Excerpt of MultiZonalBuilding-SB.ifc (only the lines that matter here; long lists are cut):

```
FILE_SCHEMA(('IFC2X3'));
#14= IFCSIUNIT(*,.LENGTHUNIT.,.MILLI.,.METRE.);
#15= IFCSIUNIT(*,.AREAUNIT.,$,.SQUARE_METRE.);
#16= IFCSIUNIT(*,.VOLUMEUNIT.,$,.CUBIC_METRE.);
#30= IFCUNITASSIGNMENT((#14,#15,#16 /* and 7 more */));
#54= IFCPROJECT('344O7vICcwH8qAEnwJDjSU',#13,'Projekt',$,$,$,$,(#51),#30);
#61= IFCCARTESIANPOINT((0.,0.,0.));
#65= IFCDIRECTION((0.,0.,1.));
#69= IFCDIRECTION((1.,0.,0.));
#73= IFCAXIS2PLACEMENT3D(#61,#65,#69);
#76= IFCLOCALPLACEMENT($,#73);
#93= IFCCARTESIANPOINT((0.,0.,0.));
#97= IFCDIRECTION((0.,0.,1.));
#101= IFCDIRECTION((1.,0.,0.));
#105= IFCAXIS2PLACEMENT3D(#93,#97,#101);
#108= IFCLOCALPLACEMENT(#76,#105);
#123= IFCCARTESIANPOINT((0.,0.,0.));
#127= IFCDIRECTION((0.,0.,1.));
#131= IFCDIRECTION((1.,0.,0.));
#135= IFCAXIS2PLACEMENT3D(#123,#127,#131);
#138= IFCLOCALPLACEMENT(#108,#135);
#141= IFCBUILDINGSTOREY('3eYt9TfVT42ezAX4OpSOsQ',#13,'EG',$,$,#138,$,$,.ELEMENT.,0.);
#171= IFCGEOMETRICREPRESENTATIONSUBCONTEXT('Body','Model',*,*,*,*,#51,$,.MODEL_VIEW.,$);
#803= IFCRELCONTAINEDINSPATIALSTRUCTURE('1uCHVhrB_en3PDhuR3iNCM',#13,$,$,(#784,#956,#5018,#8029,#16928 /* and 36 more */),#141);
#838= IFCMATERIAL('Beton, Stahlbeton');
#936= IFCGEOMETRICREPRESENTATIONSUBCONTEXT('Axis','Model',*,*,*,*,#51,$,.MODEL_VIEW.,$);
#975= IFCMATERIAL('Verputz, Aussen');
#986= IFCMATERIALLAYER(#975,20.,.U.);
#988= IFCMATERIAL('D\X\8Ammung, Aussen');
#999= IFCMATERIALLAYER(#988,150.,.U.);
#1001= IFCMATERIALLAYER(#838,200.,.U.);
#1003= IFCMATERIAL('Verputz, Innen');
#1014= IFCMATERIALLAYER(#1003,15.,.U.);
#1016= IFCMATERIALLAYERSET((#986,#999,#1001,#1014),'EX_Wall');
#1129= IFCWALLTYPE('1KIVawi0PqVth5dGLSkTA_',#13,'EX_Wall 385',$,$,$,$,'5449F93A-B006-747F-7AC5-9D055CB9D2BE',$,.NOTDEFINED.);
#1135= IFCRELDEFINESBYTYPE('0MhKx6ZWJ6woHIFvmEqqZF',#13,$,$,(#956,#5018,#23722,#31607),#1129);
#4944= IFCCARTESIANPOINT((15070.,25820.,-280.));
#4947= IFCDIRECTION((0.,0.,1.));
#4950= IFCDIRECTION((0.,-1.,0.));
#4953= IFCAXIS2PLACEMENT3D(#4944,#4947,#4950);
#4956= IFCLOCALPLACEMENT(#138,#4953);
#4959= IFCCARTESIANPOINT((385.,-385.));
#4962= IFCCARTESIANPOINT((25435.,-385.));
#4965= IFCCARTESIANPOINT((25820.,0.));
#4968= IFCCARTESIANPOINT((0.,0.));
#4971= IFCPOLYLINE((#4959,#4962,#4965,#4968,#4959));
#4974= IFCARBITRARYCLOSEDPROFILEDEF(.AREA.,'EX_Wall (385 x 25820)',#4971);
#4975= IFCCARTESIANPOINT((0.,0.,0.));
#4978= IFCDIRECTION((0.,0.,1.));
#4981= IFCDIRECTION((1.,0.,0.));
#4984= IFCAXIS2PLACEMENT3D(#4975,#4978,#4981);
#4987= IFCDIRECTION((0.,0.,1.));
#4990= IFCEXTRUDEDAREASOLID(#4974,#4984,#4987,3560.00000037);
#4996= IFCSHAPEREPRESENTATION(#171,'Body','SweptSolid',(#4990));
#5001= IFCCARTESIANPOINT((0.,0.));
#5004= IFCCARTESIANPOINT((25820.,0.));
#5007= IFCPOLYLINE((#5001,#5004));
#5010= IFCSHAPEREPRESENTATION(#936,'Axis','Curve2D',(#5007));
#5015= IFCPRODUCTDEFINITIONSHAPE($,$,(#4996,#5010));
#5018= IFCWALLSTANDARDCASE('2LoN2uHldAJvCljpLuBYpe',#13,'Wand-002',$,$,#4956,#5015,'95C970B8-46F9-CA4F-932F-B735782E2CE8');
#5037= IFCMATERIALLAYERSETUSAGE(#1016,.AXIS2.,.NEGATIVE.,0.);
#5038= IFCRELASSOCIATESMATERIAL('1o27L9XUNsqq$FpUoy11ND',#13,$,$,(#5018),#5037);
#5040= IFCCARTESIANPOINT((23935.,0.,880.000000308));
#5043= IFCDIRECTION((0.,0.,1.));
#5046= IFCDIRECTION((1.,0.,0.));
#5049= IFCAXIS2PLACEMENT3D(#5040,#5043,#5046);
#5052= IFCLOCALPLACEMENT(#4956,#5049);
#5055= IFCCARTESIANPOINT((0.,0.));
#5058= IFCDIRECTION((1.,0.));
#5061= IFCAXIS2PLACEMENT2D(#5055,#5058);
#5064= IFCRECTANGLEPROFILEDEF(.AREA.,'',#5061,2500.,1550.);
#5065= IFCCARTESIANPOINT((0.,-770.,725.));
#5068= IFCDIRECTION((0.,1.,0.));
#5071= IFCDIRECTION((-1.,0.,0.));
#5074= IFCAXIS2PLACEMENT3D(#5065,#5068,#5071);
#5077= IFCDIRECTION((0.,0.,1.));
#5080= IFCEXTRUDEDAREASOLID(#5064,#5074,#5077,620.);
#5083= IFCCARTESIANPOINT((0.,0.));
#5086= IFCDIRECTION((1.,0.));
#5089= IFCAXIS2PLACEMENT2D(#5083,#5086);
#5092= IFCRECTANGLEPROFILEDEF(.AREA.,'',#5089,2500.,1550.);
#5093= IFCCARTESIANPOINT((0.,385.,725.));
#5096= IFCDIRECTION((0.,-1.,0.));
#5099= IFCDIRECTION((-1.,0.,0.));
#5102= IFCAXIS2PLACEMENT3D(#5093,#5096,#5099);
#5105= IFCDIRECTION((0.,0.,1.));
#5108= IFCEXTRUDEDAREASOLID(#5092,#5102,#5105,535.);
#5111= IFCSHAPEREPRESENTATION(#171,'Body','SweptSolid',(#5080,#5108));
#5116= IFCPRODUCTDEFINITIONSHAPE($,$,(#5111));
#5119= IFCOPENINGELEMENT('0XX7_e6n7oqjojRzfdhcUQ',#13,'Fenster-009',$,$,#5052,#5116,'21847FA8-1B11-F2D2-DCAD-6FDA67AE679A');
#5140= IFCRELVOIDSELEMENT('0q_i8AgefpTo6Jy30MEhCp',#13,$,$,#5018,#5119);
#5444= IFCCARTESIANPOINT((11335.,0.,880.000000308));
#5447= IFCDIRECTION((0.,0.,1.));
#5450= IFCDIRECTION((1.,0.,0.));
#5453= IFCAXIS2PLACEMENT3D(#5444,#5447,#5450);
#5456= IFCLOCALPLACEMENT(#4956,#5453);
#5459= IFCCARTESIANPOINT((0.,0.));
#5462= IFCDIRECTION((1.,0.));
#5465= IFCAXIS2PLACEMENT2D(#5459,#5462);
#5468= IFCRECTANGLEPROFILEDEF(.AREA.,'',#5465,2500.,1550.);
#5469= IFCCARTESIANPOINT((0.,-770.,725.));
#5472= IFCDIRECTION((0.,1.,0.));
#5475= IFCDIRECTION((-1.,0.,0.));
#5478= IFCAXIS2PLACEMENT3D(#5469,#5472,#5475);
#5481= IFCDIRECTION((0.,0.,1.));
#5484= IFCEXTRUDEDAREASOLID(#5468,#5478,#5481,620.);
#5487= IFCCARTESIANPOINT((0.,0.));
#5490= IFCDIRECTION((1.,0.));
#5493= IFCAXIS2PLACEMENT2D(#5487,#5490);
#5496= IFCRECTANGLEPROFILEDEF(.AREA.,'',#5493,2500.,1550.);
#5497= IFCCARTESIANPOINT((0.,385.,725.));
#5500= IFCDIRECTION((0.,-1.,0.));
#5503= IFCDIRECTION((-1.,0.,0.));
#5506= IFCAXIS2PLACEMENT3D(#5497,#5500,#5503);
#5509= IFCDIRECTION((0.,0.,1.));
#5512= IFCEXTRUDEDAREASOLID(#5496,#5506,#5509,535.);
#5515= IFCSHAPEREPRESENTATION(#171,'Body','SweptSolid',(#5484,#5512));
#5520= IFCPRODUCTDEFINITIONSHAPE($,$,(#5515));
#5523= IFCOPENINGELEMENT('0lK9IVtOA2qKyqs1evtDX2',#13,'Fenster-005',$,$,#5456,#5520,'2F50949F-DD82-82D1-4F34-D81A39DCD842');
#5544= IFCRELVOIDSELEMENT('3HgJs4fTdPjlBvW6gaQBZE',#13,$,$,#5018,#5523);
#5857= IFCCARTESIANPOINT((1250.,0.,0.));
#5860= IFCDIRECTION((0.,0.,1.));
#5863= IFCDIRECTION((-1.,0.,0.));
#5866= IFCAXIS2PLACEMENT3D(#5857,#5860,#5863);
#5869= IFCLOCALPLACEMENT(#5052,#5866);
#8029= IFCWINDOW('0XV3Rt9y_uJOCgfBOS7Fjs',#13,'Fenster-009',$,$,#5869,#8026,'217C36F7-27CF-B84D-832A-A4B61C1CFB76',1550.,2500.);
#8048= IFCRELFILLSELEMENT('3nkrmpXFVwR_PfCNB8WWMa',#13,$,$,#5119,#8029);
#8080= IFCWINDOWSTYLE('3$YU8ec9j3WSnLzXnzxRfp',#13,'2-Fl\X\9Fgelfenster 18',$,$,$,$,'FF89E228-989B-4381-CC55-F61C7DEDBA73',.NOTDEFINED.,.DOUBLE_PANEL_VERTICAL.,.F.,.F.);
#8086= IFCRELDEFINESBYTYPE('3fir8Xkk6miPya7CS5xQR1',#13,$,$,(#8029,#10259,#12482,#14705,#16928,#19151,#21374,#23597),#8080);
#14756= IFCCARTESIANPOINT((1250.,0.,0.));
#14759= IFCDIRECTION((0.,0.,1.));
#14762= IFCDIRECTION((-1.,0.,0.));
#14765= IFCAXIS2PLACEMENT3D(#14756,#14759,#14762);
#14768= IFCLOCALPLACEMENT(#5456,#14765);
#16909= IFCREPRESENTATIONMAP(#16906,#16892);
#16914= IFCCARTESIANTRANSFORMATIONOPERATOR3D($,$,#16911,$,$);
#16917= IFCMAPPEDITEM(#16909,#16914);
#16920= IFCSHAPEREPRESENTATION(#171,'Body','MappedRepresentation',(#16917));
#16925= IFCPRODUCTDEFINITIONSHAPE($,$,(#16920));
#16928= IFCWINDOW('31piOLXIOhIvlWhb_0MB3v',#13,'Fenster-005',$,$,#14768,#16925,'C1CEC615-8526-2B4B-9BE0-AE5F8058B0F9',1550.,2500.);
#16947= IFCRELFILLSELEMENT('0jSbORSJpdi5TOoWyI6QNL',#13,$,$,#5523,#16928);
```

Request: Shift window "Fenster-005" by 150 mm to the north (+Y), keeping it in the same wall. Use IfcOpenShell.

```python
import ifcopenshell
import ifcopenshell.api.geometry
import ifcopenshell.util.placement

model = ifcopenshell.open("MultiZonalBuilding-SB.ifc")

window = model.by_guid("31piOLXIOhIvlWhb_0MB3v")
opening = window.FillsVoids[0].RelatingOpeningElement
wall = opening.VoidsElements[0].RelatingBuildingElement

wall_matrix = ifcopenshell.util.placement.get_local_placement(wall.ObjectPlacement)
shift = wall_matrix[:3, 0] * -150.0
before = ifcopenshell.util.placement.get_local_placement(window.ObjectPlacement)[:3, 3].copy()

# The window is placed relative to its opening, so it follows when the opening moves.
matrix = ifcopenshell.util.placement.get_local_placement(opening.ObjectPlacement)
matrix[:3, 3] += shift
ifcopenshell.api.geometry.edit_object_placement(
    model, product=opening, matrix=matrix, is_si=False, should_transform_children=True
)

after = ifcopenshell.util.placement.get_local_placement(window.ObjectPlacement)[:3, 3]
print("window moved by", (after - before).round(3) + 0.0)

model.write("MultiZonalBuilding-SB-out.ifc")
```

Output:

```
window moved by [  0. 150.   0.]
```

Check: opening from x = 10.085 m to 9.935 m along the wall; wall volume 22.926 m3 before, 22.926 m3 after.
